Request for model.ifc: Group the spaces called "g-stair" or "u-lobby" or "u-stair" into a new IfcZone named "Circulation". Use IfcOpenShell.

First a look at what the model holds.

```python
import ifcopenshell

model = ifcopenshell.open("model.ifc")
print(model.schema)
seen = {}
for space in model.by_type("IfcSpace"):
    seen[space.LongName] = seen.get(space.LongName, 0) + 1
for name, count in sorted(seen.items(), key=str):
    print(count, "x", name)
print("zones:", [z.Name for z in model.by_type("IfcZone")][:20])
```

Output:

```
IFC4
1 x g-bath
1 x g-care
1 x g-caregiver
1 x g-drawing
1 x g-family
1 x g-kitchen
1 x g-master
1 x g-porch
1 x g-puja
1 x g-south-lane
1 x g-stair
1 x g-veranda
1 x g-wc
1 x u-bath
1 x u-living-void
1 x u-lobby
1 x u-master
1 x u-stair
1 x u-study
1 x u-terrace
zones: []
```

```python
import ifcopenshell
import ifcopenshell.api.group
import ifcopenshell.api.root

model = ifcopenshell.open("model.ifc")

names = {"g-stair", "u-lobby", "u-stair"}
spaces = [s for s in model.by_type("IfcSpace") if s.LongName in names]

zone = ifcopenshell.api.root.create_entity(model, ifc_class="IfcZone", name="Circulation")
ifcopenshell.api.group.assign_group(model, products=spaces, group=zone)
print(len(spaces), "spaces in", zone.Name)

model.write("model_updated.ifc")
```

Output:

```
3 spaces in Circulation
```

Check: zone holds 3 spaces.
